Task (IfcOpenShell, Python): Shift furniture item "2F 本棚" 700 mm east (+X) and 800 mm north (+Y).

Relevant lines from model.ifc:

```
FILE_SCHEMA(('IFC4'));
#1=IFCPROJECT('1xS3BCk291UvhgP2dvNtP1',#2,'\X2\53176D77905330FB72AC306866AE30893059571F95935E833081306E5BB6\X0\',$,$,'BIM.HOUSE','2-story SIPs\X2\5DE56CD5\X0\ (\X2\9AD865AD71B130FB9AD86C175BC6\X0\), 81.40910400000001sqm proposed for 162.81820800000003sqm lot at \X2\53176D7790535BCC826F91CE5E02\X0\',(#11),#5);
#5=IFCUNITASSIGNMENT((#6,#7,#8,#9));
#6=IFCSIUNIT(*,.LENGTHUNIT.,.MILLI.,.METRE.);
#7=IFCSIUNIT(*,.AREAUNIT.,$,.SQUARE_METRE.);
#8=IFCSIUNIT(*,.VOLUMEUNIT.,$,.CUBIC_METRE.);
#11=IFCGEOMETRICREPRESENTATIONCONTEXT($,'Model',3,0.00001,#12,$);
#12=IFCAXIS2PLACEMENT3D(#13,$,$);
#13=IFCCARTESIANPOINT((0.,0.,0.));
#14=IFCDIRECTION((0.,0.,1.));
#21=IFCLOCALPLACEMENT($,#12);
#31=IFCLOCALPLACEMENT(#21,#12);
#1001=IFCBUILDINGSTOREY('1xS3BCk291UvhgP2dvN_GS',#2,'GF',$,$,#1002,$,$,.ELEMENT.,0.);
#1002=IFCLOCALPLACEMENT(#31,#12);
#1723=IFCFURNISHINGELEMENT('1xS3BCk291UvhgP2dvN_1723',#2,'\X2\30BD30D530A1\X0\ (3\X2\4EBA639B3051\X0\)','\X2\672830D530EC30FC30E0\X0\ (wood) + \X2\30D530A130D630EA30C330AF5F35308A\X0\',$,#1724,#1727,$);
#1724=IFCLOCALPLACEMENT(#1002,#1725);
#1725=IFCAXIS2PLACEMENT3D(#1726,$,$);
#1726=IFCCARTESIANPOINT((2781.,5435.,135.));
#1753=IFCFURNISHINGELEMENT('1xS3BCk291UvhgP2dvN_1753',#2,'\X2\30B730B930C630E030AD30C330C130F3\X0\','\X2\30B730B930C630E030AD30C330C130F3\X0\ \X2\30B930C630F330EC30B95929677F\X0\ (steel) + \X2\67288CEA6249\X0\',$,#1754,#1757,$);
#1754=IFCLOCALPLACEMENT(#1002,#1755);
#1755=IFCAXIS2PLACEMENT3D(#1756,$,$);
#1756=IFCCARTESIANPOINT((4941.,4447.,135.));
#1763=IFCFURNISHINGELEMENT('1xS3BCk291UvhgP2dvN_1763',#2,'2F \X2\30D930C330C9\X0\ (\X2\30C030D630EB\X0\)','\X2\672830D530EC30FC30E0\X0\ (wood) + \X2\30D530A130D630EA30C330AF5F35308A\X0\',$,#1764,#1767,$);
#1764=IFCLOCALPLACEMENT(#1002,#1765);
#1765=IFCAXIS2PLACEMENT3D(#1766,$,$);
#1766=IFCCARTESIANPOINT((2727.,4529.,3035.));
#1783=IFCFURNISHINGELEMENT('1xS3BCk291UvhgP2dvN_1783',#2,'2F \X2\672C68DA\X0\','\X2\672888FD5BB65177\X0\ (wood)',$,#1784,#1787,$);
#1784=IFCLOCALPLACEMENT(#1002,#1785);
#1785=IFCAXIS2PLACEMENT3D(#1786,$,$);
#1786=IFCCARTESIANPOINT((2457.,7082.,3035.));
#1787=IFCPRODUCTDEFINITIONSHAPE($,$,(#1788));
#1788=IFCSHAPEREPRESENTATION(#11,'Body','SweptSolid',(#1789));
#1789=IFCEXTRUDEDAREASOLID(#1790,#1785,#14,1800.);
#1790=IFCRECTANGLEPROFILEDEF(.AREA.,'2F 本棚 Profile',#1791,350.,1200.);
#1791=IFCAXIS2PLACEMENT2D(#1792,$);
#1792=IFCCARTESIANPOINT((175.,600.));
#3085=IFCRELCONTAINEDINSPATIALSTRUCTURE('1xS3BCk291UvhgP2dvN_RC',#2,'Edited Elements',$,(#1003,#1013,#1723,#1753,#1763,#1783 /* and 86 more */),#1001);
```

```python
import ifcopenshell
import ifcopenshell.api.geometry
import ifcopenshell.util.placement
import ifcopenshell.util.unit

model = ifcopenshell.open("model.ifc")
unit_scale = ifcopenshell.util.unit.calculate_unit_scale(model)

item = model.by_id(1783)
matrix = ifcopenshell.util.placement.get_local_placement(item.ObjectPlacement)
matrix[0, 3] += 0.7 / unit_scale
matrix[1, 3] += 0.8 / unit_scale
ifcopenshell.api.geometry.edit_object_placement(model, product=item, matrix=matrix, is_si=False)

print(ifcopenshell.util.placement.get_local_placement(item.ObjectPlacement).round(3) + 0.0)

model.write("model_edited.ifc")
```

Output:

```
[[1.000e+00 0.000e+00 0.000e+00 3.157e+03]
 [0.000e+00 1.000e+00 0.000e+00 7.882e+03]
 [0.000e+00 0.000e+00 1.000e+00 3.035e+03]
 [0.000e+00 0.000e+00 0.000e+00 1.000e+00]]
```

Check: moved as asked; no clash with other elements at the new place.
